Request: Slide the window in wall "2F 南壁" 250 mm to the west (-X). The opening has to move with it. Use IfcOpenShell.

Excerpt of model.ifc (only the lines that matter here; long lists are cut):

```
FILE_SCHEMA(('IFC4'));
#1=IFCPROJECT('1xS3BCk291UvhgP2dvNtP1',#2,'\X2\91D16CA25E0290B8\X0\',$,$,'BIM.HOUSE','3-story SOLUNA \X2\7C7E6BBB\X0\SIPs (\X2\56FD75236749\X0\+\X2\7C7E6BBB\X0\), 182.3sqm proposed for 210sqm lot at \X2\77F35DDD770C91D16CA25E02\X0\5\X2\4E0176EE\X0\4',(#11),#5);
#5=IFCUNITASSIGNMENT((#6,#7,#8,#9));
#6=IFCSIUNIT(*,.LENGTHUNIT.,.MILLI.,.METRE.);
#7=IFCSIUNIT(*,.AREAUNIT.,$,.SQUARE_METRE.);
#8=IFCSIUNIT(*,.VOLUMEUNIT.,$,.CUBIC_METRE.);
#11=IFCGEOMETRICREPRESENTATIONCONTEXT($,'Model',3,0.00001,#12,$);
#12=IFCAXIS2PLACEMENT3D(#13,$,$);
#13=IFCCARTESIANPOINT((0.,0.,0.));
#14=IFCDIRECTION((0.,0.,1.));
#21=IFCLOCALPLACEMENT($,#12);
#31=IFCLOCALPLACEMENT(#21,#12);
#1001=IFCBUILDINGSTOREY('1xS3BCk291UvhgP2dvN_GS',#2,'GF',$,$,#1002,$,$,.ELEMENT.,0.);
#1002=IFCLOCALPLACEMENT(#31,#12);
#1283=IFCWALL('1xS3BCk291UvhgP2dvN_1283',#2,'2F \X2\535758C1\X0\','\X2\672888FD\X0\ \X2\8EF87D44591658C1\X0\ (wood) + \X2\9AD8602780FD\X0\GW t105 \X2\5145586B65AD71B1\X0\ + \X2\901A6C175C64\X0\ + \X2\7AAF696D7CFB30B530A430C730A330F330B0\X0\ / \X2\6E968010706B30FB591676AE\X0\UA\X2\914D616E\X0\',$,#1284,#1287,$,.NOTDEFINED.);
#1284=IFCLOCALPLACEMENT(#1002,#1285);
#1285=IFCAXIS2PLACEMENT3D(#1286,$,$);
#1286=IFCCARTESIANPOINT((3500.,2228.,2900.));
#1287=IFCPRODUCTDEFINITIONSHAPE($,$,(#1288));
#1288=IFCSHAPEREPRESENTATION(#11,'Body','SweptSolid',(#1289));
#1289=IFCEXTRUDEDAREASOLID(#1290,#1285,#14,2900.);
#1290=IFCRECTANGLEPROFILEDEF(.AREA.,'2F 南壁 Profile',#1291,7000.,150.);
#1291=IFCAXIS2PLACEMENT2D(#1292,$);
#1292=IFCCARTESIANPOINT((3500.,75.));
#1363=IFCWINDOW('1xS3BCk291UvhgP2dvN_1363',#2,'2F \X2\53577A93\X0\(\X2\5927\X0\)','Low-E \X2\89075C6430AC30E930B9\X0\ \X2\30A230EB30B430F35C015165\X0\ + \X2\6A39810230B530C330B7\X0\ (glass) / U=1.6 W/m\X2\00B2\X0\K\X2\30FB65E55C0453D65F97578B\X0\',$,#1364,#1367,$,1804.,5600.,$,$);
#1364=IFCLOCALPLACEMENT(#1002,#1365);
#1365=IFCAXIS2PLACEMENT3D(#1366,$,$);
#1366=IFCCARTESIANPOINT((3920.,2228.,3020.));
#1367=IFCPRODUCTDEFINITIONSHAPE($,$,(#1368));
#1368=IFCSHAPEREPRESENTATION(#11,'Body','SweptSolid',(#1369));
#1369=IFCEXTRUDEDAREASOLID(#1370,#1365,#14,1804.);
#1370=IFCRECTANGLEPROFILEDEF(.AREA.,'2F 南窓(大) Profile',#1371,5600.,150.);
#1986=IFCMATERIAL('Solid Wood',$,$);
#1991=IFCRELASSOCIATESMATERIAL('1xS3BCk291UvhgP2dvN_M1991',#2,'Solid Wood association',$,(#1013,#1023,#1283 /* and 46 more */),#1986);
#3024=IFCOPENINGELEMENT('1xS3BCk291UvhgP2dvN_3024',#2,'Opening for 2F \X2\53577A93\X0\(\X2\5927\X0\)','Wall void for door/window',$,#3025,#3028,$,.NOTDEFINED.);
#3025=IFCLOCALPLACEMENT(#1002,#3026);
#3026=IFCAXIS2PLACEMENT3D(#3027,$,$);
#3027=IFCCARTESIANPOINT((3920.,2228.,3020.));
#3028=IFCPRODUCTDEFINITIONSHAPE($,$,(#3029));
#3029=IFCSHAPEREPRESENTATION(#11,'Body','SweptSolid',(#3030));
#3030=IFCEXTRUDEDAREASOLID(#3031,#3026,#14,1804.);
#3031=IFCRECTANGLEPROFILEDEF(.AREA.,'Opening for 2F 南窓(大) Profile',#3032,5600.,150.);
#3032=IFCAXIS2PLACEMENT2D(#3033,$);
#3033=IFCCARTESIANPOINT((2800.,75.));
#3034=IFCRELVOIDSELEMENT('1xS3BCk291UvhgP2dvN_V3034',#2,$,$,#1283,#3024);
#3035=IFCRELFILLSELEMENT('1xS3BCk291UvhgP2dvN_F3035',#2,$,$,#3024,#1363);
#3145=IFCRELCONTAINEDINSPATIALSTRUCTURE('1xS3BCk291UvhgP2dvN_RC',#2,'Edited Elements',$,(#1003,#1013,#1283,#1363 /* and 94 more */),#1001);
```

```python
import ifcopenshell
import ifcopenshell.api.geometry
import ifcopenshell.util.placement
import ifcopenshell.util.unit

model = ifcopenshell.open("model.ifc")
unit_scale = ifcopenshell.util.unit.calculate_unit_scale(model)

window = model.by_guid("1xS3BCk291UvhgP2dvN_1363")
opening = window.FillsVoids[0].RelatingOpeningElement
wall = opening.VoidsElements[0].RelatingBuildingElement

wall_matrix = ifcopenshell.util.placement.get_local_placement(wall.ObjectPlacement)
shift = wall_matrix[:3, 0] * -0.25 / unit_scale
before = ifcopenshell.util.placement.get_local_placement(window.ObjectPlacement)[:3, 3].copy()

# The window is not placed relative to its opening, so move both.
for product in (opening, window):
    matrix = ifcopenshell.util.placement.get_local_placement(product.ObjectPlacement)
    matrix[:3, 3] += shift
    ifcopenshell.api.geometry.edit_object_placement(model, product=product, matrix=matrix, is_si=False)

after = ifcopenshell.util.placement.get_local_placement(window.ObjectPlacement)[:3, 3]
print("window moved by", (after - before).round(3) + 0.0)

model.write("model-out.ifc")
```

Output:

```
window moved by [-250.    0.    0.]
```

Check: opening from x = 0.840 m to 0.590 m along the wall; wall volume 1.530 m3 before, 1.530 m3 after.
